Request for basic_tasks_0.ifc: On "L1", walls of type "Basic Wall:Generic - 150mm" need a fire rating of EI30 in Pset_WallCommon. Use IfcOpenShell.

First a look at what the model holds.

```python
import ifcopenshell
import ifcopenshell.util.element

model = ifcopenshell.open("basic_tasks_0.ifc")
print(model.schema)
storey = next(s for s in model.by_type("IfcBuildingStorey") if s.Name == "L1")
walls = [e for e in ifcopenshell.util.element.get_decomposition(storey) if e.is_a("IfcWall")]
seen = {}
for e in walls:
    element_type = ifcopenshell.util.element.get_type(e)
    key = (element_type.Name if element_type != e and element_type else None, ifcopenshell.util.element.get_pset(e, "Pset_WallCommon", "FireRating"))
    seen[key] = seen.get(key, 0) + 1
for (name, value), count in sorted(seen.items(), key=str):
    print(count, "x", name, "|", value)
```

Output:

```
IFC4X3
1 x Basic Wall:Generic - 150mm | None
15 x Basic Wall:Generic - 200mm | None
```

```python
import ifcopenshell
import ifcopenshell.api.pset
import ifcopenshell.util.element

model = ifcopenshell.open("basic_tasks_0.ifc")

storey = next(s for s in model.by_type("IfcBuildingStorey") if s.Name == "L1")
walls = [e for e in ifcopenshell.util.element.get_decomposition(storey) if e.is_a("IfcWall")]

count = 0
for e in walls:
    element_type = ifcopenshell.util.element.get_type(e)
    if element_type in (None, e) or element_type.Name != "Basic Wall:Generic - 150mm":
        continue
    # add_pset returns the element's existing set when there is one.
    pset = ifcopenshell.api.pset.add_pset(model, product=e, name="Pset_WallCommon")
    ifcopenshell.api.pset.edit_pset(model, pset=pset, properties={"FireRating": "EI30"})
    count += 1

print(count, "walls updated")

model.write("basic_tasks_0_updated.ifc")
```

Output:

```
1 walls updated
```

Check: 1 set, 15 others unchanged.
